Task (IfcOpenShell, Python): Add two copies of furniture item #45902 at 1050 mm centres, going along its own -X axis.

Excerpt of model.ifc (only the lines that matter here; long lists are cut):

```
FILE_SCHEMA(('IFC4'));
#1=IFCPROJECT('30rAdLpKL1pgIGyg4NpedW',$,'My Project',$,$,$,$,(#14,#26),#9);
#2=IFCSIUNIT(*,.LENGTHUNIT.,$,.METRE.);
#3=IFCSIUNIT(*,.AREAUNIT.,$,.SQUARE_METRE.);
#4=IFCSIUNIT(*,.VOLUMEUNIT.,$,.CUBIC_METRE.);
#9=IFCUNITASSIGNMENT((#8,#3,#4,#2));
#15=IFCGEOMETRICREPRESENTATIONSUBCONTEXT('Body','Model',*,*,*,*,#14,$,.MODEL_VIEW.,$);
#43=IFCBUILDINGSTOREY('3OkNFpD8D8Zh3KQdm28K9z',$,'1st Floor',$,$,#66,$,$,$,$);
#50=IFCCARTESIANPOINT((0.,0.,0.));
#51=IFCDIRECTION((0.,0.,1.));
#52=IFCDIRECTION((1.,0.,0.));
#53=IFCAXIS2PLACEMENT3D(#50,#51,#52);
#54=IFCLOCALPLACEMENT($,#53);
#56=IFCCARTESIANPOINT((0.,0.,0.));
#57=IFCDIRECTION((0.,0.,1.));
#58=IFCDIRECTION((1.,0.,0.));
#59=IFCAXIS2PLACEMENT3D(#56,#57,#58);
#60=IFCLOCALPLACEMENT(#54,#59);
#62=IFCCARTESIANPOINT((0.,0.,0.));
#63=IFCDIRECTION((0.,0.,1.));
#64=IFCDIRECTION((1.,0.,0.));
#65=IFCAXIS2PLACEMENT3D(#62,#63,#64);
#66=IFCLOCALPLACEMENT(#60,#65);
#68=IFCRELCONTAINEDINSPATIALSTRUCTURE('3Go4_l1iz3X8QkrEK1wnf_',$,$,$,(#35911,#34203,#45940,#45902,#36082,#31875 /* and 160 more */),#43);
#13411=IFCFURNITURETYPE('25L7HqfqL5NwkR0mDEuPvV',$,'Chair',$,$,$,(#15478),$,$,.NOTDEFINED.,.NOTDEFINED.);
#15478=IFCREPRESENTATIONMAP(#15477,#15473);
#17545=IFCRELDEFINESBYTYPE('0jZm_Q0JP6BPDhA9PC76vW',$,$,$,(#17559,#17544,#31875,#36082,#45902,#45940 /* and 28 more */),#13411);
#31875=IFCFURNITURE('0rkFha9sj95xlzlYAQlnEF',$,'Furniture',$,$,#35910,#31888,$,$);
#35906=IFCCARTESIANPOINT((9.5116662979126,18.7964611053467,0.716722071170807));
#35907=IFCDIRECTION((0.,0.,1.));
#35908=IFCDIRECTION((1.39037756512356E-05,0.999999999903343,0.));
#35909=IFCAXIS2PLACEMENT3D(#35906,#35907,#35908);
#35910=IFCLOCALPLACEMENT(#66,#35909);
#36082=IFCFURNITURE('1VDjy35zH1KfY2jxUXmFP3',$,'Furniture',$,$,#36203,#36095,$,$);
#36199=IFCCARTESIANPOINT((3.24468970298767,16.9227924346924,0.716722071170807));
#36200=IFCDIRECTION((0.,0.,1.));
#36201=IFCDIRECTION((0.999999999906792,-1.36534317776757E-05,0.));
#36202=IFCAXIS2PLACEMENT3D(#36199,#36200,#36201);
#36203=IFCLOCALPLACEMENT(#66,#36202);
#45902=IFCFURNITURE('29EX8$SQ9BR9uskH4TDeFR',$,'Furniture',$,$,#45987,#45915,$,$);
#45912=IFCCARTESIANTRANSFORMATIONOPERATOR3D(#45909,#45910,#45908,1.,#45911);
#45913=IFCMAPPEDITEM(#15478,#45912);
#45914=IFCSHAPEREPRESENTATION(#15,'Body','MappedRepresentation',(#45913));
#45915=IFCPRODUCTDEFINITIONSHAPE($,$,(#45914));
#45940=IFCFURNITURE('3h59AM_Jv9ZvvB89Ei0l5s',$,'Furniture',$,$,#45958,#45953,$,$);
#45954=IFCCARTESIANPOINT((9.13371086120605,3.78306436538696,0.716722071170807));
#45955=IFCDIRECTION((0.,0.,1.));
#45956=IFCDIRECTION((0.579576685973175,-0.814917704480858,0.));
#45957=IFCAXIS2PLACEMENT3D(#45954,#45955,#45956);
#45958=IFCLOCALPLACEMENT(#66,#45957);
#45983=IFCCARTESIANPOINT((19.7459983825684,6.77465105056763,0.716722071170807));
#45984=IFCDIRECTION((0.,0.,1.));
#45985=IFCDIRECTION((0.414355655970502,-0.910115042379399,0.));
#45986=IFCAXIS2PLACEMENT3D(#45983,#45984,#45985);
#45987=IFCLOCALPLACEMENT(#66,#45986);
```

```python
import ifcopenshell
import ifcopenshell.api.geometry
import ifcopenshell.api.root
import ifcopenshell.util.element
import ifcopenshell.util.placement

model = ifcopenshell.open("model.ifc")

source = model.by_guid("29EX8$SQ9BR9uskH4TDeFR")
base = ifcopenshell.util.placement.get_local_placement(source.ObjectPlacement)
step = -base[:3, 0] * 1.05

for i in range(1, 3):
    copy = ifcopenshell.api.root.copy_class(model, product=source)
    copy.Representation = ifcopenshell.util.element.copy_deep(
        model, source.Representation, exclude=["IfcGeometricRepresentationContext", "IfcRepresentationMap"]
    )
    matrix = base.copy()
    matrix[:3, 3] += i * step
    print("added at", matrix[:3, 3].round(3) + 0.0)
    ifcopenshell.api.geometry.edit_object_placement(model, product=copy, matrix=matrix, is_si=False)

model.write("model_edited.ifc")
```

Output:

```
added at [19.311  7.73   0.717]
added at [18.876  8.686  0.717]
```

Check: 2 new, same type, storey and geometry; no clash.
